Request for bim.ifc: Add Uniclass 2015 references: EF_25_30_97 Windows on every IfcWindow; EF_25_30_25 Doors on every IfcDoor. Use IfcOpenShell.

First a look at what the model holds.

```python
import ifcopenshell

model = ifcopenshell.open("bim.ifc")
print(model.schema)
print("classifications:", [c.Name for c in model.by_type("IfcClassification")])
for ifc_class in ("IfcDoor", "IfcRoof", "IfcStair", "IfcWall", "IfcWindow"):
    print(ifc_class, len(model.by_type(ifc_class)))
```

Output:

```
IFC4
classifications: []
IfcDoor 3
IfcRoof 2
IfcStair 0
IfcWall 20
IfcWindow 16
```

```python
import ifcopenshell
import ifcopenshell.api.classification

model = ifcopenshell.open("bim.ifc")

system = ifcopenshell.api.classification.add_classification(model, classification="Uniclass 2015")

codes = {
    "IfcWindow": ("EF_25_30_97", "Windows"),
    "IfcDoor": ("EF_25_30_25", "Doors"),
}
for ifc_class, (code, name) in codes.items():
    products = model.by_type(ifc_class)
    ifcopenshell.api.classification.add_reference(
        model, products=products, classification=system, identification=code, name=name
    )
    print(code, len(products))

model.write("bim-out.ifc")
```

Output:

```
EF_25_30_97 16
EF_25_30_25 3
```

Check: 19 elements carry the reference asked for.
